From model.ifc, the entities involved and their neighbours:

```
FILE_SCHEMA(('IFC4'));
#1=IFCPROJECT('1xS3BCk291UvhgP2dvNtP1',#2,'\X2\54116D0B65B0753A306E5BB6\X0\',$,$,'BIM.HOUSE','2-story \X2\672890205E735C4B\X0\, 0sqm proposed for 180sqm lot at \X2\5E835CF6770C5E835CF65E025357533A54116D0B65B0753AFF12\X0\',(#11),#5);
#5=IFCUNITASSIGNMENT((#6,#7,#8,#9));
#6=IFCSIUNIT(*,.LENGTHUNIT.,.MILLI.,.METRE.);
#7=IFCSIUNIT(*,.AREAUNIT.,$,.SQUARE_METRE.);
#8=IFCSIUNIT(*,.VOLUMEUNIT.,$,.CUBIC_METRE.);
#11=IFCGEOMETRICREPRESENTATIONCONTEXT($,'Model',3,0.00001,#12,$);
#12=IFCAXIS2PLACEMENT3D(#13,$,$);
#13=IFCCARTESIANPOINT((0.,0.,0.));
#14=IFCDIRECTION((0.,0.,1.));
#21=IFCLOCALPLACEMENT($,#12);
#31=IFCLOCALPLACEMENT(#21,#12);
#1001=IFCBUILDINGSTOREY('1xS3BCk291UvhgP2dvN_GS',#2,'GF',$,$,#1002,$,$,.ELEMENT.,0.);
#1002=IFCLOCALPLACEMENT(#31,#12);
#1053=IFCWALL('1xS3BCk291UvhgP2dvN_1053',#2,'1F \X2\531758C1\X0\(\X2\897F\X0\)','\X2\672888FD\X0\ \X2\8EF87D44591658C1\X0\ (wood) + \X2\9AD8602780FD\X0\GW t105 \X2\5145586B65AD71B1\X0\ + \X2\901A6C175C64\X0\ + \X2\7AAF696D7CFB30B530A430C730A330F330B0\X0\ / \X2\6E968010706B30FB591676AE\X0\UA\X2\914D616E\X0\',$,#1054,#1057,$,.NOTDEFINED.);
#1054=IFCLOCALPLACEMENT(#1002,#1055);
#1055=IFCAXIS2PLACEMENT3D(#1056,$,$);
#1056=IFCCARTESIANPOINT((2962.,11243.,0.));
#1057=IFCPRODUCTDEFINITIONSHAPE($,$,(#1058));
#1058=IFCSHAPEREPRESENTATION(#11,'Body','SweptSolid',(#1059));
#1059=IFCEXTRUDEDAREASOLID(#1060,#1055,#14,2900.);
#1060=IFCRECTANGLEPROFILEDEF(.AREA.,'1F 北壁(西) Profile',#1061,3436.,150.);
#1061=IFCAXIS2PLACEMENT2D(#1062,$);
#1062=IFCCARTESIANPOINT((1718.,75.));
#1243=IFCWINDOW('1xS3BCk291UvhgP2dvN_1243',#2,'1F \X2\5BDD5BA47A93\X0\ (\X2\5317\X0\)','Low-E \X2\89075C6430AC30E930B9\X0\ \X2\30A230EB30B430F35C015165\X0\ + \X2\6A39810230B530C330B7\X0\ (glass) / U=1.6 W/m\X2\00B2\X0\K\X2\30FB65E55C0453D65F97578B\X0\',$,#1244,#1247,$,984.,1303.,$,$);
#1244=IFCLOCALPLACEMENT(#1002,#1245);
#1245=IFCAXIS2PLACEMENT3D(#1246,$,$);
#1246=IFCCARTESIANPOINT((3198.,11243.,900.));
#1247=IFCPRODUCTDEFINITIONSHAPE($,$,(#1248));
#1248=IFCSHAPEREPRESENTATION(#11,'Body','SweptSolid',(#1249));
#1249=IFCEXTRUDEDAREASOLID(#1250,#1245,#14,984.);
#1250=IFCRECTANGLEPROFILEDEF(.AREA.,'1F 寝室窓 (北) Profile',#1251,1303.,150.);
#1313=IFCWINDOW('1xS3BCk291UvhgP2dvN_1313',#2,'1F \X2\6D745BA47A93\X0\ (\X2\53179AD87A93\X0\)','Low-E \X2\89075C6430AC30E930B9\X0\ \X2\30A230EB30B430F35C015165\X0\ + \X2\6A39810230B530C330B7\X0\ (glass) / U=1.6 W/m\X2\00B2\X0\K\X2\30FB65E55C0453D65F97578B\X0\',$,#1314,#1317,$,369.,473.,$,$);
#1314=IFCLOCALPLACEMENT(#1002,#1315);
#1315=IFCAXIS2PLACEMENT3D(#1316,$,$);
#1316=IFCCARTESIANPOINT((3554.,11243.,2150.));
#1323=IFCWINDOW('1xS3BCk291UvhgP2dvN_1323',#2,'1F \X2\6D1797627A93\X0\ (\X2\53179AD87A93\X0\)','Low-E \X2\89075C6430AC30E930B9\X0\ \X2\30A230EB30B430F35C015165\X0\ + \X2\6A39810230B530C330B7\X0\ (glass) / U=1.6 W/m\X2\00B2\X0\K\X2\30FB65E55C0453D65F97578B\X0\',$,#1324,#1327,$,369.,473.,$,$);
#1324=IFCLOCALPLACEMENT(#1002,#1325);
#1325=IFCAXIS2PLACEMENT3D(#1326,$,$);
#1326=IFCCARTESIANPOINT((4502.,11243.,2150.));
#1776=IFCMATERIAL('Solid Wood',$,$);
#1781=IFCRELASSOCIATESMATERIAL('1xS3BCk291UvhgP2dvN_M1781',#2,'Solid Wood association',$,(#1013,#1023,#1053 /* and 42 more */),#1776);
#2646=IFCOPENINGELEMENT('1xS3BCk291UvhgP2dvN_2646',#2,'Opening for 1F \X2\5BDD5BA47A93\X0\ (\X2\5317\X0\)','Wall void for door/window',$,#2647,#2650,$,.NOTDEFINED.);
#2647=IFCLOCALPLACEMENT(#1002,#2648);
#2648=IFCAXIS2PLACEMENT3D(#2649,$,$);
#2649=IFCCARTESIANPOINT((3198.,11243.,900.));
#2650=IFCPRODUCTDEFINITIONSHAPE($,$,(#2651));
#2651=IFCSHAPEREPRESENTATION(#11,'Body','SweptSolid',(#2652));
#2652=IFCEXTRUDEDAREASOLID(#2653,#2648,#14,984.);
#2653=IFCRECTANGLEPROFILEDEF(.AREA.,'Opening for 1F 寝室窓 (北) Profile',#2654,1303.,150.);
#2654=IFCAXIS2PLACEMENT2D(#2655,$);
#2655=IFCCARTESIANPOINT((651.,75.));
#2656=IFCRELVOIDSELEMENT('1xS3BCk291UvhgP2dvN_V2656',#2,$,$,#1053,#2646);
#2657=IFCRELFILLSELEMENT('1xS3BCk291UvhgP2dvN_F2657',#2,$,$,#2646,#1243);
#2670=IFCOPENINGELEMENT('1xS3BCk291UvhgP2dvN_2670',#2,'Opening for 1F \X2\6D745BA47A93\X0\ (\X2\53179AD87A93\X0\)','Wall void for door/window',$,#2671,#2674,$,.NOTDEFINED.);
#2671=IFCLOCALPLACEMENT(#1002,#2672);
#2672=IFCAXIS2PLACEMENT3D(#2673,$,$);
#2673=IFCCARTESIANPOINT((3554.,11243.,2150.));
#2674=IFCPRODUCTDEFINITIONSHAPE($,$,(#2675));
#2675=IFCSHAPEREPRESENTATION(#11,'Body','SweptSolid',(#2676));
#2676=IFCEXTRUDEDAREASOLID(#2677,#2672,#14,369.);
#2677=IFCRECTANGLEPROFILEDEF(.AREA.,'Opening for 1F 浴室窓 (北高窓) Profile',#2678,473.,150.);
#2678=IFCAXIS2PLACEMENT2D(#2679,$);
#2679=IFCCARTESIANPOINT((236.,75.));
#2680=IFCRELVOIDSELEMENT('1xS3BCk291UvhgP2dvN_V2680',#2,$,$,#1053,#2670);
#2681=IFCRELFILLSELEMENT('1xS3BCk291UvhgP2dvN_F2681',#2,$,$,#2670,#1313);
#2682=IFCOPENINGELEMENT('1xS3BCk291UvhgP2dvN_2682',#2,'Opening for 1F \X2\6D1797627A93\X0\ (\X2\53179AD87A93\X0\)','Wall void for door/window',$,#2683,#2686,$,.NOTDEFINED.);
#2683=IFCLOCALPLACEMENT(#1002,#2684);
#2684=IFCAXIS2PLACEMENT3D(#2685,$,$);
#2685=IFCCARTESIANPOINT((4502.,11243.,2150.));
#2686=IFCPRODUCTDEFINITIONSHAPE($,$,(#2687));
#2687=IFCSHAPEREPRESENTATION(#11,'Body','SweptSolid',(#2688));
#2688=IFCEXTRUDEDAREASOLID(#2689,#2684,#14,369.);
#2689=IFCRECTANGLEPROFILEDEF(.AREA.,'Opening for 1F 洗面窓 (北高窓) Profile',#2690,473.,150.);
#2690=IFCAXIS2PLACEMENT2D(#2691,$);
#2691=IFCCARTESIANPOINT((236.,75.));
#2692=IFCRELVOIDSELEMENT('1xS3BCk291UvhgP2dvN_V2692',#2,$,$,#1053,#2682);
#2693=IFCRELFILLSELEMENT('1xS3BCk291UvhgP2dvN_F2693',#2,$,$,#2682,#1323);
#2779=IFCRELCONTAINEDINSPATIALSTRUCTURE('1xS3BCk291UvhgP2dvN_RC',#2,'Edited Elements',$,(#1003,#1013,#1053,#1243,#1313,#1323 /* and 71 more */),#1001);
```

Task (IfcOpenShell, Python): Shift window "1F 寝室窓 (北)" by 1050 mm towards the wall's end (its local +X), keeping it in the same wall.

```python
import ifcopenshell
import ifcopenshell.api.geometry
import ifcopenshell.util.placement

model = ifcopenshell.open("model.ifc")

window = model.by_id(1243)
opening = window.FillsVoids[0].RelatingOpeningElement
wall = opening.VoidsElements[0].RelatingBuildingElement

wall_matrix = ifcopenshell.util.placement.get_local_placement(wall.ObjectPlacement)
shift = wall_matrix[:3, 0] * 1050.0
before = ifcopenshell.util.placement.get_local_placement(window.ObjectPlacement)[:3, 3].copy()

# The window is not placed relative to its opening, so move both.
for product in (opening, window):
    matrix = ifcopenshell.util.placement.get_local_placement(product.ObjectPlacement)
    matrix[:3, 3] += shift
    ifcopenshell.api.geometry.edit_object_placement(model, product=product, matrix=matrix, is_si=False)

after = ifcopenshell.util.placement.get_local_placement(window.ObjectPlacement)[:3, 3]
print("window moved by", (after - before).round(3) + 0.0)

model.write("model_updated.ifc")
```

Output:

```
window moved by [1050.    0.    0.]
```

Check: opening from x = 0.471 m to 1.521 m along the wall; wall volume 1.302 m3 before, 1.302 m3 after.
